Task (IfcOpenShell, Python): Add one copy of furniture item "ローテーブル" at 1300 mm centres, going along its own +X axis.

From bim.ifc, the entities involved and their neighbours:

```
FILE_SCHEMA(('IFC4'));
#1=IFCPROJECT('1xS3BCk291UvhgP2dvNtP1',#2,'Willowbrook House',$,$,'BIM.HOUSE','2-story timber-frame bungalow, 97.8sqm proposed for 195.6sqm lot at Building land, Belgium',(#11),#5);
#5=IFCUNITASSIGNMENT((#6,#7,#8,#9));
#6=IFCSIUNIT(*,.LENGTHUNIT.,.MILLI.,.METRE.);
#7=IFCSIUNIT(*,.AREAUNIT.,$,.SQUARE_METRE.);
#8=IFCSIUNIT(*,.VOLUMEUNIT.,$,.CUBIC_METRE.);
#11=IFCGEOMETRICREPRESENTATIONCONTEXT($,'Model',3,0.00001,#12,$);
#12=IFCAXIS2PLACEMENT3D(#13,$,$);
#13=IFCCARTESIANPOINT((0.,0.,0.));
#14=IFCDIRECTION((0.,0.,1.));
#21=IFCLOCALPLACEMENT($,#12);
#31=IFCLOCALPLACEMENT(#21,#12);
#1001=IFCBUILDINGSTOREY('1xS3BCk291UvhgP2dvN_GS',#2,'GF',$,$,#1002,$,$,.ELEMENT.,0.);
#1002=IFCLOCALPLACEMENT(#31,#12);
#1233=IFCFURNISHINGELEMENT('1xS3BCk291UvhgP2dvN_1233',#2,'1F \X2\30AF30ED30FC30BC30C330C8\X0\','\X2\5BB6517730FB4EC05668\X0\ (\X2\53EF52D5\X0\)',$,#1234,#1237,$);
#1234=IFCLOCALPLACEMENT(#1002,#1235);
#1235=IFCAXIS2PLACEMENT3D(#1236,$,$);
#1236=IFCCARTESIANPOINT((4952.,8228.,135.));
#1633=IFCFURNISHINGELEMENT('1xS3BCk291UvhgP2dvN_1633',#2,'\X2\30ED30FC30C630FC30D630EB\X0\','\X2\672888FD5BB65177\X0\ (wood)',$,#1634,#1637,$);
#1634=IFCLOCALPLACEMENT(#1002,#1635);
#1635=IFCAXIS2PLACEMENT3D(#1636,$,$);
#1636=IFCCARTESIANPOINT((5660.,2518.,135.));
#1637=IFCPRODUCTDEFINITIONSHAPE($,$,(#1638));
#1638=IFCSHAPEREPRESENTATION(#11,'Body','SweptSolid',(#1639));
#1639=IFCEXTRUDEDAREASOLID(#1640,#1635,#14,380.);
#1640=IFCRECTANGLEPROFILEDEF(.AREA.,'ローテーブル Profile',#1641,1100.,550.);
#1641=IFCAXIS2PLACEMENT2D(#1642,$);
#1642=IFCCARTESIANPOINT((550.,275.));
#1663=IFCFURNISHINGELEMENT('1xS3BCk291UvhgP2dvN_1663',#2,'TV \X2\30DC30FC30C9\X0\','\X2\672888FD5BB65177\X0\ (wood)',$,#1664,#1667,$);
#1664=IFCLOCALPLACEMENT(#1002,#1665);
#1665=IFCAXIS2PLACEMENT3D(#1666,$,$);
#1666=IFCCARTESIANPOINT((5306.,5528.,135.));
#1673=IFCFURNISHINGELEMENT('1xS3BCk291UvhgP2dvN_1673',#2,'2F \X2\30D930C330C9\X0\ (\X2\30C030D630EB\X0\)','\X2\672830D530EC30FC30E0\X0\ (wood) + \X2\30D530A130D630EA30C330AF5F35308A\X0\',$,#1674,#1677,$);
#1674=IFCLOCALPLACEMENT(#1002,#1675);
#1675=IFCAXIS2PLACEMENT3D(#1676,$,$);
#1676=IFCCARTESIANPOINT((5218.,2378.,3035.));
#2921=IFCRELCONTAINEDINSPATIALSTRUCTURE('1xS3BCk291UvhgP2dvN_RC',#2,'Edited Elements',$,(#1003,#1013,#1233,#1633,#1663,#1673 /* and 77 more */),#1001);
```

```python
import ifcopenshell
import ifcopenshell.api.geometry
import ifcopenshell.api.root
import ifcopenshell.util.element
import ifcopenshell.util.placement
import ifcopenshell.util.unit

model = ifcopenshell.open("bim.ifc")
unit_scale = ifcopenshell.util.unit.calculate_unit_scale(model)


def reuse_history(source, copy):
    """copy_class also copies each property set's owner history, people and application; keep the originals."""
    for rel in copy.IsDefinedBy:
        if rel.is_a("IfcRelDefinesByProperties") and (history := rel.RelatingPropertyDefinition.OwnerHistory):
            rel.RelatingPropertyDefinition.OwnerHistory = source.OwnerHistory
            ifcopenshell.util.element.remove_deep2(model, history)


source = model.by_id(1633)
base = ifcopenshell.util.placement.get_local_placement(source.ObjectPlacement)
step = base[:3, 0] * 1.3 / unit_scale

for i in range(1, 2):
    copy = ifcopenshell.api.root.copy_class(model, product=source)
    copy.Representation = ifcopenshell.util.element.copy_deep(
        model, source.Representation, exclude=["IfcGeometricRepresentationContext", "IfcRepresentationMap"]
    )
    reuse_history(source, copy)
    matrix = base.copy()
    matrix[:3, 3] += i * step
    print("added at", matrix[:3, 3].round(3) + 0.0)
    ifcopenshell.api.geometry.edit_object_placement(model, product=copy, matrix=matrix, is_si=False)

model.write("bim_edited.ifc")
```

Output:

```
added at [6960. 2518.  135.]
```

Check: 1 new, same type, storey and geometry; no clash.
